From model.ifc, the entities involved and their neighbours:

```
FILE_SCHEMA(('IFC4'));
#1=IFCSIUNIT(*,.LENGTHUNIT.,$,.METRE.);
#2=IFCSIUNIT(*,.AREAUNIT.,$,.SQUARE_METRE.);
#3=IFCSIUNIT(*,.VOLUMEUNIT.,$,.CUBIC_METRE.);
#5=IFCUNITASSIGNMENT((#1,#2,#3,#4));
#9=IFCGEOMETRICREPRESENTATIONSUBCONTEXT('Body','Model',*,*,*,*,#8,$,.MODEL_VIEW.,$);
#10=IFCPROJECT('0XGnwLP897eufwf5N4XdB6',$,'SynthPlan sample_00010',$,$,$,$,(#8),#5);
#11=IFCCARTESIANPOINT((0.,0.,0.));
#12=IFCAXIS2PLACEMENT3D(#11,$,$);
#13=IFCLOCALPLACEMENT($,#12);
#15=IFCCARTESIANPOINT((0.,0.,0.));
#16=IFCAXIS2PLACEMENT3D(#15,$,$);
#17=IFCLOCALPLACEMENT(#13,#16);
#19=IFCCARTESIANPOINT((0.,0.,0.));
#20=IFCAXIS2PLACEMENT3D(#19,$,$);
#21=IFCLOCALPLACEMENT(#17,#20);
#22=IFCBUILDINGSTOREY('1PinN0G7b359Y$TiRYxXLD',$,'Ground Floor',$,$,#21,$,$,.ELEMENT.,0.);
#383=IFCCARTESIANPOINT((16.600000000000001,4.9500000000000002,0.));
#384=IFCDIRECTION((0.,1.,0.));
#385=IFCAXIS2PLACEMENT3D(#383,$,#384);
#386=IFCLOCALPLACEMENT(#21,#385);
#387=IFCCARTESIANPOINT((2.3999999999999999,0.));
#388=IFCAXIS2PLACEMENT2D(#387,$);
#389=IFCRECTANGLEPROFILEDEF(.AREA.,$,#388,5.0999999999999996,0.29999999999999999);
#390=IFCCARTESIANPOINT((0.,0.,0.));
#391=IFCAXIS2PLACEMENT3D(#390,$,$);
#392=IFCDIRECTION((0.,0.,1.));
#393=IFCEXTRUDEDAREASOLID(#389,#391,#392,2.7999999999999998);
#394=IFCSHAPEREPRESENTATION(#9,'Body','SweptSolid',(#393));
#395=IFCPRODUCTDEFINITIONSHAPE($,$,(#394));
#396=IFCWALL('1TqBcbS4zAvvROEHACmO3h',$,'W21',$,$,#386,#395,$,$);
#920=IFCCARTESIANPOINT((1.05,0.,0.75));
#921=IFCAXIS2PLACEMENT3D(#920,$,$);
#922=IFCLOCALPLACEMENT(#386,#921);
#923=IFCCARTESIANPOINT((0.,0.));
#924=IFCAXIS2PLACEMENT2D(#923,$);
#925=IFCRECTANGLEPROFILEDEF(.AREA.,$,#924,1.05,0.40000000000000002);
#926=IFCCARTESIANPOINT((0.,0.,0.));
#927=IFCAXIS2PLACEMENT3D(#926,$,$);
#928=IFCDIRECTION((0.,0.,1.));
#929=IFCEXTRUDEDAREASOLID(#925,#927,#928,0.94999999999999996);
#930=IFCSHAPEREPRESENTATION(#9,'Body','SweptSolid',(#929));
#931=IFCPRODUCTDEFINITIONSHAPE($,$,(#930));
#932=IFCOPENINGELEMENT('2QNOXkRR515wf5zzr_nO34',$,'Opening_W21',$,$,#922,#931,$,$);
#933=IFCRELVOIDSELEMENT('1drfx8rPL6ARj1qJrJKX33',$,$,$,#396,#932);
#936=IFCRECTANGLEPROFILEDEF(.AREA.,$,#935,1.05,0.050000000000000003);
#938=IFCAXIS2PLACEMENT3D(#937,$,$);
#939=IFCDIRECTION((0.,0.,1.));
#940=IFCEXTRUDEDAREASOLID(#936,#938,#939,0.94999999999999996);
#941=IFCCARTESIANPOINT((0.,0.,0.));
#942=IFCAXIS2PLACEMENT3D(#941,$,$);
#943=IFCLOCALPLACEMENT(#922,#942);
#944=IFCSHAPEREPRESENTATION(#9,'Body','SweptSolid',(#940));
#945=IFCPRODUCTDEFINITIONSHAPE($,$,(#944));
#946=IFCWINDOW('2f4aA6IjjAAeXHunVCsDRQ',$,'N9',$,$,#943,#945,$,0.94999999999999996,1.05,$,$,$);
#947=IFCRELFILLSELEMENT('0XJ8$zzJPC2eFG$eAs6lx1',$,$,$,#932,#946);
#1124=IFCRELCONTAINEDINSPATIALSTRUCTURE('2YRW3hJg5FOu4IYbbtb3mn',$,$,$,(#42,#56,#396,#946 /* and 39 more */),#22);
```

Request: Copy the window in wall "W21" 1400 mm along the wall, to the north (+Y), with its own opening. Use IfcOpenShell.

```python
import ifcopenshell
import ifcopenshell.api.feature
import ifcopenshell.api.geometry
import ifcopenshell.api.root
import ifcopenshell.geom
import ifcopenshell.util.element
import ifcopenshell.util.placement
import ifcopenshell.util.shape

model = ifcopenshell.open("model.ifc")
settings = ifcopenshell.geom.settings()


def volume(element):
    """Net volume in cubic metres, openings subtracted."""
    shape = ifcopenshell.geom.create_shape(settings, element)
    return ifcopenshell.util.shape.get_volume(shape.geometry)


window = model.by_id(946)
opening = window.FillsVoids[0].RelatingOpeningElement
wall = opening.VoidsElements[0].RelatingBuildingElement
before = volume(wall)
shift = ifcopenshell.util.placement.get_local_placement(wall.ObjectPlacement)[:3, 0] * 1.4

# copy_class copies the void relationship, type, container and properties, but no geometry.
new_opening = ifcopenshell.api.root.copy_class(model, product=opening)
new_opening.Representation = ifcopenshell.util.element.copy_deep(
    model, opening.Representation, exclude=["IfcGeometricRepresentationContext", "IfcRepresentationMap"]
)
new_window = ifcopenshell.api.root.copy_class(model, product=window)
new_window.Representation = ifcopenshell.util.element.copy_deep(
    model, window.Representation, exclude=["IfcGeometricRepresentationContext", "IfcRepresentationMap"]
)
ifcopenshell.api.feature.add_filling(model, opening=new_opening, element=new_window)

for old, new in ((opening, new_opening), (window, new_window)):
    matrix = ifcopenshell.util.placement.get_local_placement(old.ObjectPlacement)
    matrix[:3, 3] += shift
    ifcopenshell.api.geometry.edit_object_placement(model, product=new, matrix=matrix, is_si=False)

after = volume(wall)

print(f"wall volume {before:.3f} -> {after:.3f} m3")

model.write("model_rev.ifc")
```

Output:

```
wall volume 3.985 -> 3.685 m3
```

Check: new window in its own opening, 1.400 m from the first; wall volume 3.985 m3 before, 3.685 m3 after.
